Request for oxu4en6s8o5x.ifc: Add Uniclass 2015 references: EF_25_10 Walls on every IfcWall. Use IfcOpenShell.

First a look at what the model holds.

```python
import ifcopenshell

model = ifcopenshell.open("oxu4en6s8o5x.ifc")
print(model.schema)
print("classifications:", [c.Name for c in model.by_type("IfcClassification")])
for ifc_class in ("IfcDoor", "IfcRoof", "IfcStair", "IfcWall", "IfcWindow"):
    print(ifc_class, len(model.by_type(ifc_class)))
```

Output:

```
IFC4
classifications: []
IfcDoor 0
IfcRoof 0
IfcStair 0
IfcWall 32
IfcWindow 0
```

```python
import ifcopenshell
import ifcopenshell.api.classification

model = ifcopenshell.open("oxu4en6s8o5x.ifc")

system = ifcopenshell.api.classification.add_classification(model, classification="Uniclass 2015")

codes = {
    "IfcWall": ("EF_25_10", "Walls"),
}
for ifc_class, (code, name) in codes.items():
    products = model.by_type(ifc_class)
    ifcopenshell.api.classification.add_reference(
        model, products=products, classification=system, identification=code, name=name
    )
    print(code, len(products))

model.write("oxu4en6s8o5x_rev.ifc")
```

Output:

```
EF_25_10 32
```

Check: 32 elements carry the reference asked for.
